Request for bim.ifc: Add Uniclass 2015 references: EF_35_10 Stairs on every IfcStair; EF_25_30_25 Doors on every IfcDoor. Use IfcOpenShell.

First a look at what the model holds.

```python
import ifcopenshell

model = ifcopenshell.open("bim.ifc")
print(model.schema)
print("classifications:", [c.Name for c in model.by_type("IfcClassification")])
for ifc_class in ("IfcDoor", "IfcRoof", "IfcStair", "IfcWall", "IfcWindow"):
    print(ifc_class, len(model.by_type(ifc_class)))
```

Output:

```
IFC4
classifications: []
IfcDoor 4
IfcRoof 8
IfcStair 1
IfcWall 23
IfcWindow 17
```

```python
import ifcopenshell
import ifcopenshell.api.classification

model = ifcopenshell.open("bim.ifc")

system = ifcopenshell.api.classification.add_classification(model, classification="Uniclass 2015")

codes = {
    "IfcStair": ("EF_35_10", "Stairs"),
    "IfcDoor": ("EF_25_30_25", "Doors"),
}
for ifc_class, (code, name) in codes.items():
    products = model.by_type(ifc_class)
    ifcopenshell.api.classification.add_reference(
        model, products=products, classification=system, identification=code, name=name
    )
    print(code, len(products))

model.write("bim_updated.ifc")
```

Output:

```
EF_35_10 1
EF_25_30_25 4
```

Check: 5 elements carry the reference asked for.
